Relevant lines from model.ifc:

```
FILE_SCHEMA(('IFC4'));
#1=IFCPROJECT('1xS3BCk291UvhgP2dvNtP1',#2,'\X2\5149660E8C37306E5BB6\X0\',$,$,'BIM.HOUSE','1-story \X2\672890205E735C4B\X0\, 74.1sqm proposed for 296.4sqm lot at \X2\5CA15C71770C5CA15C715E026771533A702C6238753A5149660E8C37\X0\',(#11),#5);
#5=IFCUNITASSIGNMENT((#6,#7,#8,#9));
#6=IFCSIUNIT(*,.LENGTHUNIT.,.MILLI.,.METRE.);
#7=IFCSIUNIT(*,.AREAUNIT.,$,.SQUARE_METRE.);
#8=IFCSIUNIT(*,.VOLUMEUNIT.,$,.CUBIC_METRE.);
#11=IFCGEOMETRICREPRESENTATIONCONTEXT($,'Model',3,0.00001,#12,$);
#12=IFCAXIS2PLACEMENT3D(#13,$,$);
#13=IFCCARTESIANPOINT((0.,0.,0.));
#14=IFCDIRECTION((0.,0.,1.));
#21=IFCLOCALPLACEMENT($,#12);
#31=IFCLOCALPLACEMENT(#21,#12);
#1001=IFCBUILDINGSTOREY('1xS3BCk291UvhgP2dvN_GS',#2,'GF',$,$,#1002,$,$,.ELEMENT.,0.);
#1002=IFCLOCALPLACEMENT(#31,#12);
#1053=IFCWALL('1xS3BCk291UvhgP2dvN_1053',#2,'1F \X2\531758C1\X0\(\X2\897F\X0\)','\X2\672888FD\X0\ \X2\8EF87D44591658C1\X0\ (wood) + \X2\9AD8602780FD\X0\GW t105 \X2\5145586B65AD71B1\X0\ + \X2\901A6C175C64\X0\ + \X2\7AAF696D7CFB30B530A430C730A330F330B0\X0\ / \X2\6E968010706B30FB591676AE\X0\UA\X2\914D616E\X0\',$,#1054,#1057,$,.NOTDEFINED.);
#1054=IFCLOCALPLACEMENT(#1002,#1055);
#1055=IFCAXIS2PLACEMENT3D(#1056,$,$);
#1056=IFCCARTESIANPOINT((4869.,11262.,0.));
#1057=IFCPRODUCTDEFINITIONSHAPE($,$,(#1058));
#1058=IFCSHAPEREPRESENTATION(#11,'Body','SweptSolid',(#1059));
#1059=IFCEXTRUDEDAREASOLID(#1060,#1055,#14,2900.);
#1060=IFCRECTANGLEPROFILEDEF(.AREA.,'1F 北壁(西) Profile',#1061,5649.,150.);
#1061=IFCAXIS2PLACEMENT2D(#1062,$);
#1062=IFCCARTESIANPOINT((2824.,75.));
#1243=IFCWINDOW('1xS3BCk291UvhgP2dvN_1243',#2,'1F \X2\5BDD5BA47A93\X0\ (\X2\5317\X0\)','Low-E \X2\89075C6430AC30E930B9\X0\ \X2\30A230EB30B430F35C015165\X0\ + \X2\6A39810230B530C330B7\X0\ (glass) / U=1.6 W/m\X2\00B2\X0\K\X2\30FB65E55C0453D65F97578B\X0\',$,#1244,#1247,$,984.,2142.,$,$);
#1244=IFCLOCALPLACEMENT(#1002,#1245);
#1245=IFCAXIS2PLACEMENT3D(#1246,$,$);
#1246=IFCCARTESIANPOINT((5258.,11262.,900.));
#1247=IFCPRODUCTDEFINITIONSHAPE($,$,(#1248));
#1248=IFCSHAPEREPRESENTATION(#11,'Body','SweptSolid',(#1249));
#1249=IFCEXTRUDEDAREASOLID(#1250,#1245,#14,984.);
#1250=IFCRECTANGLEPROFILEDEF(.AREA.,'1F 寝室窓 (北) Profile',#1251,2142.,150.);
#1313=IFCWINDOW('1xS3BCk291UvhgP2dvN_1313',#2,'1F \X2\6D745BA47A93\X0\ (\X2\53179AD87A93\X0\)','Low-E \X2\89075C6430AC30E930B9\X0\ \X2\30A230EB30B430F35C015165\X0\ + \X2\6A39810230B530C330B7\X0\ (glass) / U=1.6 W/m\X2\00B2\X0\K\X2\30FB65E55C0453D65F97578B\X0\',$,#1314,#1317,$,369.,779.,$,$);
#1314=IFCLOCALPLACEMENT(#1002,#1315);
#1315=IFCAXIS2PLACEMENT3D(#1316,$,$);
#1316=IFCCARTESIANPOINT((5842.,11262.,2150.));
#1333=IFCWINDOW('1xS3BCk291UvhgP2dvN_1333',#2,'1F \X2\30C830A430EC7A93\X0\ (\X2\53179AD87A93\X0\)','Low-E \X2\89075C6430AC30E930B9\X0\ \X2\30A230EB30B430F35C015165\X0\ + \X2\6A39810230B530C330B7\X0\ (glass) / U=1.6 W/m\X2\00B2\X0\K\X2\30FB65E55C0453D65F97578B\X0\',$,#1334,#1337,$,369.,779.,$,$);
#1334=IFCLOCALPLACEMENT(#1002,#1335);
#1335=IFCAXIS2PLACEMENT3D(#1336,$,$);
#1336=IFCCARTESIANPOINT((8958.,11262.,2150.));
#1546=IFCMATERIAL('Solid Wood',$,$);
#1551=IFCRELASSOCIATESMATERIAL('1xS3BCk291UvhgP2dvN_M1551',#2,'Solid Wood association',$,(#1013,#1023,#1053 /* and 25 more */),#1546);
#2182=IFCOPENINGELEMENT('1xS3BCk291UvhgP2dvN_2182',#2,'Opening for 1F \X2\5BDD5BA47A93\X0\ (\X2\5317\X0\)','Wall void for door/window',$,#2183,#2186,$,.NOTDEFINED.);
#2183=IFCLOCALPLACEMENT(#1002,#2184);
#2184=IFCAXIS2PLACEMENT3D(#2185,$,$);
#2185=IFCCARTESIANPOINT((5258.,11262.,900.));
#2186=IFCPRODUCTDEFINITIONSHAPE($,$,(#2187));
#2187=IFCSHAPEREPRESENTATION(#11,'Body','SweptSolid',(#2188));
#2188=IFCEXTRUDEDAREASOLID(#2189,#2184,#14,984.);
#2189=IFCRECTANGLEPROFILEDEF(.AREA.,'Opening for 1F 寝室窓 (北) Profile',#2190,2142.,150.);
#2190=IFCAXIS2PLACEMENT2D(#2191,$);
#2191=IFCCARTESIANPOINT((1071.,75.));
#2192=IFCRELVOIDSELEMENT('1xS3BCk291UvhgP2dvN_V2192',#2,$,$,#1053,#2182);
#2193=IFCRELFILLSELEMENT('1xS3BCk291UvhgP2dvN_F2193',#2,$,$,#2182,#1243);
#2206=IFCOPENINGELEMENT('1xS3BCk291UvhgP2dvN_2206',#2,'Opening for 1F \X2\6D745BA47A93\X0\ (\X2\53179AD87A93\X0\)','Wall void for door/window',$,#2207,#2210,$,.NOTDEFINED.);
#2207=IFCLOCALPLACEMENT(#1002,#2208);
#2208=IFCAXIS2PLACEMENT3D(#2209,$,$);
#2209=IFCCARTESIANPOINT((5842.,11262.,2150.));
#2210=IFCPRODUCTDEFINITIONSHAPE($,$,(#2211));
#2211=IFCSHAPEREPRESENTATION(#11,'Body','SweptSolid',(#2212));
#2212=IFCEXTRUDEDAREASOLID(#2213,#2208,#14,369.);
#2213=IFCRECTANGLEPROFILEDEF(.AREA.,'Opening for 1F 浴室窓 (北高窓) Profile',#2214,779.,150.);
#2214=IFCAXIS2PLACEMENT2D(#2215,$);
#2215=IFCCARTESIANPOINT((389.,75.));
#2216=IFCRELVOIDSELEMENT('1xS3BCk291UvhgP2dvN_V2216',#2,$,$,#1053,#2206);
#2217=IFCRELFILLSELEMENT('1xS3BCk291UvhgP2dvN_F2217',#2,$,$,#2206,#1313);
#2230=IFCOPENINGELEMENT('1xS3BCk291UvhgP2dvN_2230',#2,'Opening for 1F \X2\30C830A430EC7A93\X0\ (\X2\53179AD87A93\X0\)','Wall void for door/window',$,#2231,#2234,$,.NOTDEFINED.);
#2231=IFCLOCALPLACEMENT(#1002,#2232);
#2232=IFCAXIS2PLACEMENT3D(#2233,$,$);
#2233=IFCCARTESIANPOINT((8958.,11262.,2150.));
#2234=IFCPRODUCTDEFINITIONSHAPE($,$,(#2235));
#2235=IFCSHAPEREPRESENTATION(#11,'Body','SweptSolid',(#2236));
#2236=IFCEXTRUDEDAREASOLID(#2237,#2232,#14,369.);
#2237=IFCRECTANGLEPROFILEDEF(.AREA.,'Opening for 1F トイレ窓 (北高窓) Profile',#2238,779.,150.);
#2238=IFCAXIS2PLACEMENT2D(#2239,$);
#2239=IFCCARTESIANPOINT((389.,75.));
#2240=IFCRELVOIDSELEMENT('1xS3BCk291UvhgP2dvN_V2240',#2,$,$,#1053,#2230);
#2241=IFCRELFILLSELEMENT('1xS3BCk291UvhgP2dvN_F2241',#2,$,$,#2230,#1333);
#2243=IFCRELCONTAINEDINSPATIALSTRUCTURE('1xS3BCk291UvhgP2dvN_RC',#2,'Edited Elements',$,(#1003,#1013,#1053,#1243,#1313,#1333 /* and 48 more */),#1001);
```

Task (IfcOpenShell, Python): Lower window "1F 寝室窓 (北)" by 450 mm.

```python
import numpy as np
import ifcopenshell
import ifcopenshell.api.geometry
import ifcopenshell.util.placement
import ifcopenshell.util.unit

model = ifcopenshell.open("model.ifc")
unit_scale = ifcopenshell.util.unit.calculate_unit_scale(model)

window = model.by_id(1243)
opening = window.FillsVoids[0].RelatingOpeningElement
dz = -0.45 / unit_scale

shift = np.array([0.0, 0.0, dz])
# The window is not placed relative to its opening, so move both.
for product in (opening, window):
    matrix = ifcopenshell.util.placement.get_local_placement(product.ObjectPlacement)
    matrix[:3, 3] += shift
    ifcopenshell.api.geometry.edit_object_placement(model, product=product, matrix=matrix, is_si=False)

print(f"moved by {dz * unit_scale:+.3f} m")

model.write("model_edited.ifc")
```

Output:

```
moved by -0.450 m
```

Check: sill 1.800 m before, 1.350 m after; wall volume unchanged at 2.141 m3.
